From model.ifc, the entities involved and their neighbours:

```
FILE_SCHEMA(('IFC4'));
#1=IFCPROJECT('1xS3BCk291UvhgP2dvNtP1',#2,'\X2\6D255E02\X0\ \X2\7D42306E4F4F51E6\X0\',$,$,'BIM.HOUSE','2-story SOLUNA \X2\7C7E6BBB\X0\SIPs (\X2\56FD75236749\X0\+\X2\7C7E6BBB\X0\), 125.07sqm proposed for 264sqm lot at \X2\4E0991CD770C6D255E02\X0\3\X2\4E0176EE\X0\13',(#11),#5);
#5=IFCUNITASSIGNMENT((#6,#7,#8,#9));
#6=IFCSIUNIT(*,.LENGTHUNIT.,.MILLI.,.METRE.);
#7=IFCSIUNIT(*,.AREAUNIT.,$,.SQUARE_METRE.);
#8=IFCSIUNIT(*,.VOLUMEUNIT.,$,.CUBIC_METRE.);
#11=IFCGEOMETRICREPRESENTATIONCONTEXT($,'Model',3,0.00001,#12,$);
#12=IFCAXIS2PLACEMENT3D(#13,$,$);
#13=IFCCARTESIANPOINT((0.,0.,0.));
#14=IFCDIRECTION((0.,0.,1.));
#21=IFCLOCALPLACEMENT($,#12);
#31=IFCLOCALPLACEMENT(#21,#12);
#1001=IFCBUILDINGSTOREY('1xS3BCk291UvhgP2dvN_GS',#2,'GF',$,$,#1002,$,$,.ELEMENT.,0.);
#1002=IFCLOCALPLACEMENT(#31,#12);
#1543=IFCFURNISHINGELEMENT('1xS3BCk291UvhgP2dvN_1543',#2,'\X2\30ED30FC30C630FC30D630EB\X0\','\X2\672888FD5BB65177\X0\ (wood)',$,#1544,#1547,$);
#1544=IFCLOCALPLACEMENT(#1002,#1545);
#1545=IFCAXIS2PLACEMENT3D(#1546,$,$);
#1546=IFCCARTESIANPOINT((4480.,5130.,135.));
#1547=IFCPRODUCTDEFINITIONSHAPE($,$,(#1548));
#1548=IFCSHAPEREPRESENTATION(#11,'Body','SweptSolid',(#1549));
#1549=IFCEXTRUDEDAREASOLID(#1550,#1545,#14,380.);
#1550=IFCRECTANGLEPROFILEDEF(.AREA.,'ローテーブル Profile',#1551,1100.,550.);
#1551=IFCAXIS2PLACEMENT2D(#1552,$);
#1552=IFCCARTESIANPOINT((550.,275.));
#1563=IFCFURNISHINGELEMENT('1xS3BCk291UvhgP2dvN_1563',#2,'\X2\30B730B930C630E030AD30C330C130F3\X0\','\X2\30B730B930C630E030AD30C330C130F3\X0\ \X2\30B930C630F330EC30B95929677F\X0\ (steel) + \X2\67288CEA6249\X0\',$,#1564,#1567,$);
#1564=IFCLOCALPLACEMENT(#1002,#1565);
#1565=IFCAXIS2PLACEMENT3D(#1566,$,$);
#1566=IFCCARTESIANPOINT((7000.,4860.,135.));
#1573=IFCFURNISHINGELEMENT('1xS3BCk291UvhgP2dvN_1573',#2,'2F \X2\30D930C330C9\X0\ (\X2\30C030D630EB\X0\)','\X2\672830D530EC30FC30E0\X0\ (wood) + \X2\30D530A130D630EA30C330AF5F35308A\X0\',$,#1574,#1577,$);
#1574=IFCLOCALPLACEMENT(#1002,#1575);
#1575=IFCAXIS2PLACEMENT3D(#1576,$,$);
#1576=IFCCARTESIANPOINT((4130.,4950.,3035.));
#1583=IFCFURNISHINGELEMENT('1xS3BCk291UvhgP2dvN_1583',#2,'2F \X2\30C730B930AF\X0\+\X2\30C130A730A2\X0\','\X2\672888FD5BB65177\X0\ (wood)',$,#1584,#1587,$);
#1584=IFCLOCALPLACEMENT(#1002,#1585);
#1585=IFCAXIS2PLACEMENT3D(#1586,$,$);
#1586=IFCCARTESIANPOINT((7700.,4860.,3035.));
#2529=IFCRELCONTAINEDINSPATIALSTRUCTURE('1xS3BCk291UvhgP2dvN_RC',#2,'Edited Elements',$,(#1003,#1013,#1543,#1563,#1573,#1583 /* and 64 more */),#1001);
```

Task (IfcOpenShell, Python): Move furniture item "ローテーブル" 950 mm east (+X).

```python
import ifcopenshell
import ifcopenshell.api.geometry
import ifcopenshell.util.placement

model = ifcopenshell.open("model.ifc")

item = model.by_guid("1xS3BCk291UvhgP2dvN_1543")
matrix = ifcopenshell.util.placement.get_local_placement(item.ObjectPlacement)
matrix[0, 3] += 950.0
ifcopenshell.api.geometry.edit_object_placement(model, product=item, matrix=matrix, is_si=False)

print(ifcopenshell.util.placement.get_local_placement(item.ObjectPlacement).round(3) + 0.0)

model.write("model-out.ifc")
```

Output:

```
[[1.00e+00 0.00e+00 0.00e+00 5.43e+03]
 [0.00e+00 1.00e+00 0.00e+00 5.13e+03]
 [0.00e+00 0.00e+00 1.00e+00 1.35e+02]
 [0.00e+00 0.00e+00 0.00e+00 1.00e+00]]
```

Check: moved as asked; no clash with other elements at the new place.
